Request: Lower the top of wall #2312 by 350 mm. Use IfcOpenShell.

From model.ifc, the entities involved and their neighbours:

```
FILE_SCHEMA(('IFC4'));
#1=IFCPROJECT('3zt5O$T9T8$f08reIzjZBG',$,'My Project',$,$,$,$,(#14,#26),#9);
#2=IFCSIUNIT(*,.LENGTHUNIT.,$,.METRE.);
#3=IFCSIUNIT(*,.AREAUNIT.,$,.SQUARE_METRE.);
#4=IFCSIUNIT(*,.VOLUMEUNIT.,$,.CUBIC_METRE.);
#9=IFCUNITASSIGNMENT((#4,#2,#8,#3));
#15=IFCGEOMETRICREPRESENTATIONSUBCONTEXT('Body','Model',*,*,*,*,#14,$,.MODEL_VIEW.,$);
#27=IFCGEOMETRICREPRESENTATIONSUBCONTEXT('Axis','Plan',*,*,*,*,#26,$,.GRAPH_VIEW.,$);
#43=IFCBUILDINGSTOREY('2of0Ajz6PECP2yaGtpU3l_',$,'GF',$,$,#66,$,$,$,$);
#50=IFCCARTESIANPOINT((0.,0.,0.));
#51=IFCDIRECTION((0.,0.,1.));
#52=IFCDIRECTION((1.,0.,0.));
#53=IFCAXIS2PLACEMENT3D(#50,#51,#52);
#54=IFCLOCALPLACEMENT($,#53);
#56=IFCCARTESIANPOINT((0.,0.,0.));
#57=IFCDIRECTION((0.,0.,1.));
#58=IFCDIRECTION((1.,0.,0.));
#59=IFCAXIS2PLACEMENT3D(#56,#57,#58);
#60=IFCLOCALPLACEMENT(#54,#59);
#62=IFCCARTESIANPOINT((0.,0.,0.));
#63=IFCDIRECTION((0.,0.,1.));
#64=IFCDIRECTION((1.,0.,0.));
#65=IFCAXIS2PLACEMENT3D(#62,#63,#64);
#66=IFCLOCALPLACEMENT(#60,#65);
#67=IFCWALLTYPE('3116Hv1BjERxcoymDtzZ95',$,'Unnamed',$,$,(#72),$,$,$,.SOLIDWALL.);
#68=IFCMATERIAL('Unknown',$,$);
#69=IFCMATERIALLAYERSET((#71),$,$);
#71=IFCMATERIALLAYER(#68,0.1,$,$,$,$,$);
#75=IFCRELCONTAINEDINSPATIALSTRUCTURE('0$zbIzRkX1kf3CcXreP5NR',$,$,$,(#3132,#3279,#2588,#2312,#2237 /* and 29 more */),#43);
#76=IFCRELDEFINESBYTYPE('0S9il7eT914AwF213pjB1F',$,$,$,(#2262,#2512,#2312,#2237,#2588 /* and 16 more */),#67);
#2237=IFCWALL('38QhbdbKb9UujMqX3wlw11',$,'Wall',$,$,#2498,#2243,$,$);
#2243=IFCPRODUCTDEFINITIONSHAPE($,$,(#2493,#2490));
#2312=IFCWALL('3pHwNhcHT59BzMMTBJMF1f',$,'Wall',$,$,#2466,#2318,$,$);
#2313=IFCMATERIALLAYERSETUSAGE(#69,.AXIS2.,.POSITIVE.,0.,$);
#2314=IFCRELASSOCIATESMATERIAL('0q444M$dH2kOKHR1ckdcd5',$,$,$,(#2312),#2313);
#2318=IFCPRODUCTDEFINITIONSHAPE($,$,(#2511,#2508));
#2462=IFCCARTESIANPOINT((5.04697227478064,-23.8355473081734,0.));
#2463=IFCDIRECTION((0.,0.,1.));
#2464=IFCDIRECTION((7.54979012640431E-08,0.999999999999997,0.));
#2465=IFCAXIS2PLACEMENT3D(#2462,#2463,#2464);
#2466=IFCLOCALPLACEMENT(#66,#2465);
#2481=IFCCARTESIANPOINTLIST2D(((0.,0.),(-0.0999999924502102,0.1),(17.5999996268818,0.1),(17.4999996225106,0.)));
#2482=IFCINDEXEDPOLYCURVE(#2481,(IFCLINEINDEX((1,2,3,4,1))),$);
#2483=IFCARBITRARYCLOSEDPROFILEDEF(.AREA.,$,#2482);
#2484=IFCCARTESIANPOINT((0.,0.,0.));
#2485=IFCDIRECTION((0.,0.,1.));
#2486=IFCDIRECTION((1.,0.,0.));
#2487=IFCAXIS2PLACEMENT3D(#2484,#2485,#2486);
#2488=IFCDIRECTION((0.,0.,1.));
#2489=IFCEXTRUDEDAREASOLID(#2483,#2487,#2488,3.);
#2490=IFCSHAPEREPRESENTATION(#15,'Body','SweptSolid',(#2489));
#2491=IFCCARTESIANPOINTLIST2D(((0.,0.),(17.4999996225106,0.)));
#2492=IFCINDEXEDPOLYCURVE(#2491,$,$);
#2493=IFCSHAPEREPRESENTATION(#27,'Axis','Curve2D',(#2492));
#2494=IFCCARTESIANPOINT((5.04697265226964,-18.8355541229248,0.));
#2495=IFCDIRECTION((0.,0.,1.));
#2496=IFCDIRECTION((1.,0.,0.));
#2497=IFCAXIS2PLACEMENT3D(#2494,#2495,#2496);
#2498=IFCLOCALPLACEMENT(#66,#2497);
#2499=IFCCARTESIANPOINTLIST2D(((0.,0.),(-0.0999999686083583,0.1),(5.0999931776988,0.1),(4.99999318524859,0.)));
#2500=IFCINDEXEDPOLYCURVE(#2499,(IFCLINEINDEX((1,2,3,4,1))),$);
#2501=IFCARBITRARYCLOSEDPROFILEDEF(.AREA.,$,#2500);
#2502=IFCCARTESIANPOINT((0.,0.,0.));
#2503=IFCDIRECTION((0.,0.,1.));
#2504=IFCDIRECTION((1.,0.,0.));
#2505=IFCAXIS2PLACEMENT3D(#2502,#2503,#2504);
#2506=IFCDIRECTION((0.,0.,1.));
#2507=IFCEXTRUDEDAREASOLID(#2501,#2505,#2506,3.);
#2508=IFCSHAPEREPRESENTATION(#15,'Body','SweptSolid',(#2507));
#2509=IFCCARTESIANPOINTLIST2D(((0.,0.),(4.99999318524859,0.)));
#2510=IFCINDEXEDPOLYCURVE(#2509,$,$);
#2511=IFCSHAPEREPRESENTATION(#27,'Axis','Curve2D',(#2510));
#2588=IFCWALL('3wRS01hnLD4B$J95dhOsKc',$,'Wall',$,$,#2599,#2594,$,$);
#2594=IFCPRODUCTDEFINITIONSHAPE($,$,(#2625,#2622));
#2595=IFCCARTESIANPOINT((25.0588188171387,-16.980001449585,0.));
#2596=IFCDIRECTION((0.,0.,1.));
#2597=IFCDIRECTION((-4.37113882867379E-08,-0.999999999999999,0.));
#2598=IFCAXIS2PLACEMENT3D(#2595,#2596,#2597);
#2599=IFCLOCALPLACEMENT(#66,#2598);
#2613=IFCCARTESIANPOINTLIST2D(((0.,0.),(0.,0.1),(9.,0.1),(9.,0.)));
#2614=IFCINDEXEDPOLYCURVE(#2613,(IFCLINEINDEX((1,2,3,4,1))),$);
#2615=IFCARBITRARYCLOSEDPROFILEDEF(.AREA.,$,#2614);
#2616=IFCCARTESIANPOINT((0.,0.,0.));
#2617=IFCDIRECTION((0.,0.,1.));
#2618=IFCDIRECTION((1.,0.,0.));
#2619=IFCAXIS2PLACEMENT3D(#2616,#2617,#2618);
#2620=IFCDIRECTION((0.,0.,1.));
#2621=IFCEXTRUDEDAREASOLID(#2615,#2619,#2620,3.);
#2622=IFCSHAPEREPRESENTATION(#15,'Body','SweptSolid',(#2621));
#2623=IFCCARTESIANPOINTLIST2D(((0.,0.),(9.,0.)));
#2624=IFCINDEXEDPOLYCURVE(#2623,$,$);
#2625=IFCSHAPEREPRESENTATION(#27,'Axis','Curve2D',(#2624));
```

```python
import ifcopenshell
import ifcopenshell.geom
import ifcopenshell.util.representation
import ifcopenshell.util.shape

model = ifcopenshell.open("model.ifc")
settings = ifcopenshell.geom.settings()


def volume(element):
    """Net volume in cubic metres, openings subtracted."""
    shape = ifcopenshell.geom.create_shape(settings, element)
    return ifcopenshell.util.shape.get_volume(shape.geometry)


wall = model.by_guid("3pHwNhcHT59BzMMTBJMF1f")
before = volume(wall)

body = ifcopenshell.util.representation.get_representation(wall, "Model", "Body")
solid = body.Items[0]
old_height = solid.Depth
solid.Depth -= 0.35
after = volume(wall)

print(f"height {old_height:g} -> {solid.Depth:g}, volume {before:.3f} -> {after:.3f} m3")

model.write("model_rev.ifc")
```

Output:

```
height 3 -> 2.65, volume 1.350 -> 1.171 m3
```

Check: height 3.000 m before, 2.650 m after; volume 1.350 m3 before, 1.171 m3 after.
